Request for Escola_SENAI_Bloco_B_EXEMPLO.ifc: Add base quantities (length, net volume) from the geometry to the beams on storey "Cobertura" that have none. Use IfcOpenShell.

First a look at what the model holds.

```python
import ifcopenshell
import ifcopenshell.util.element
import ifcopenshell.util.unit

model = ifcopenshell.open("Escola_SENAI_Bloco_B_EXEMPLO.ifc")
print(model.schema)
for unit_type in ("LENGTHUNIT", "AREAUNIT", "VOLUMEUNIT"):
    print(unit_type, ifcopenshell.util.unit.calculate_unit_scale(model, unit_type))
storey = next(s for s in model.by_type("IfcBuildingStorey") if s.Name == "Cobertura")
beams = [e for e in ifcopenshell.util.element.get_decomposition(storey) if e.is_a("IfcBeam")]
for e in sorted(beams, key=lambda e: e.id()):
    print(e.id(), e.is_a(), e.Name, list(ifcopenshell.util.element.get_psets(e, qtos_only=True)), sep=" | ")
```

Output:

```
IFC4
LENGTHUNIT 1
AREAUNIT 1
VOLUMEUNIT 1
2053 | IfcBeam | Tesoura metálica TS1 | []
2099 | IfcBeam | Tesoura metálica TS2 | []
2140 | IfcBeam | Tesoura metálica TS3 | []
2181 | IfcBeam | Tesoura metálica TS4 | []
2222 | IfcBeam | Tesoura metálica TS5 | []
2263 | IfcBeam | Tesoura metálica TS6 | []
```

```python
import ifcopenshell
import ifcopenshell.api.pset
import ifcopenshell.geom
import ifcopenshell.util.element
import ifcopenshell.util.shape
import ifcopenshell.util.unit

model = ifcopenshell.open("Escola_SENAI_Bloco_B_EXEMPLO.ifc")
unit_scale = ifcopenshell.util.unit.calculate_unit_scale(model)
volume_scale = ifcopenshell.util.unit.calculate_unit_scale(model, "VOLUMEUNIT")
settings = ifcopenshell.geom.settings()

storey = next(s for s in model.by_type("IfcBuildingStorey") if s.Name == "Cobertura")
beams = [e for e in ifcopenshell.util.element.get_decomposition(storey) if e.is_a("IfcBeam")]

for e in sorted(beams, key=lambda e: e.id()):
    if ifcopenshell.util.element.get_psets(e, qtos_only=True, should_inherit=False):
        continue
    # Geometry comes back in metres, in the element's own axes.
    shape = ifcopenshell.geom.create_shape(settings, e)
    values = {
        "Length": ifcopenshell.util.shape.get_max_xyz(shape.geometry) / unit_scale,
        "NetVolume": ifcopenshell.util.shape.get_volume(shape.geometry) / volume_scale,
    }
    qto = ifcopenshell.api.pset.add_qto(model, product=e, name="Qto_BeamBaseQuantities")
    ifcopenshell.api.pset.edit_qto(model, qto=qto, properties=values)
    print(e.id(), {k: round(v, 3) for k, v in values.items()})

model.write("Escola_SENAI_Bloco_B_EXEMPLO_v2.ifc")
```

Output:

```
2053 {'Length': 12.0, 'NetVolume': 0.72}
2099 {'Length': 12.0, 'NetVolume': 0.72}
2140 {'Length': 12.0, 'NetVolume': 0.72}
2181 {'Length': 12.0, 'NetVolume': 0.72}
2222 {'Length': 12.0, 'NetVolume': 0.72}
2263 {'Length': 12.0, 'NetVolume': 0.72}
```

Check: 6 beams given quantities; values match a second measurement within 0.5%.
